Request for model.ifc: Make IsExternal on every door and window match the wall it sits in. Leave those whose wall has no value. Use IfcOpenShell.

First a look at what the model holds.

```python
import ifcopenshell
import ifcopenshell.util.element

model = ifcopenshell.open("model.ifc")
print(model.schema)
seen = {}
for e in model.by_type("IfcDoor") + model.by_type("IfcWindow"):
    if not e.FillsVoids:
        continue
    host = e.FillsVoids[0].RelatingOpeningElement.VoidsElements[0].RelatingBuildingElement
    own = ifcopenshell.util.element.get_pset(e, f"Pset_{e.is_a()[3:].removesuffix('StandardCase')}Common", "IsExternal")
    wall = ifcopenshell.util.element.get_pset(host, "Pset_WallCommon", "IsExternal")
    seen[e.is_a(), own, wall] = seen.get((e.is_a(), own, wall), 0) + 1
for (cls, own, wall), count in sorted(seen.items(), key=str):
    print(count, cls, "IsExternal:", own, "| host wall:", wall)
```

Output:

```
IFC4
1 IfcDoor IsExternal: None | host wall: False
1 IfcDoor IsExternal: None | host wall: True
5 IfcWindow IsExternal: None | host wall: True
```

```python
import ifcopenshell
import ifcopenshell.api.pset
import ifcopenshell.util.element

model = ifcopenshell.open("model.ifc")

count = 0
for ifc_class, pset_name in (("IfcDoor", "Pset_DoorCommon"), ("IfcWindow", "Pset_WindowCommon")):
    for e in model.by_type(ifc_class):
        if not e.FillsVoids:
            continue
        host = e.FillsVoids[0].RelatingOpeningElement.VoidsElements[0].RelatingBuildingElement
        external = ifcopenshell.util.element.get_pset(host, "Pset_WallCommon", "IsExternal")
        if external is None or ifcopenshell.util.element.get_pset(e, pset_name, "IsExternal") == external:
            continue
        pset = ifcopenshell.api.pset.add_pset(model, product=e, name=pset_name)
        ifcopenshell.api.pset.edit_pset(model, pset=pset, properties={"IsExternal": external})
        count += 1

print(count, "updated")

model.write("model_v2.ifc")
```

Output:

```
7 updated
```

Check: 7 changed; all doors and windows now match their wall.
